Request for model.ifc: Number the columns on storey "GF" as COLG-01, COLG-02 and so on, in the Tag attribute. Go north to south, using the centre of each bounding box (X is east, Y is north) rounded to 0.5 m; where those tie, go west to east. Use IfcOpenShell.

First a look at what the model holds.

```python
import ifcopenshell
import ifcopenshell.util.element
import ifcopenshell.util.placement

model = ifcopenshell.open("model.ifc")
print(model.schema)
storey = next(s for s in model.by_type("IfcBuildingStorey") if s.Name == "GF")
columns = [e for e in ifcopenshell.util.element.get_decomposition(storey) if e.is_a("IfcColumn")]
for e in sorted(columns, key=lambda e: e.id()):
    origin = ifcopenshell.util.placement.get_local_placement(e.ObjectPlacement)[:3, 3]
    print(e.id(), e.Tag, e.Name, origin.round(2) + 0.0, sep=" | ")
```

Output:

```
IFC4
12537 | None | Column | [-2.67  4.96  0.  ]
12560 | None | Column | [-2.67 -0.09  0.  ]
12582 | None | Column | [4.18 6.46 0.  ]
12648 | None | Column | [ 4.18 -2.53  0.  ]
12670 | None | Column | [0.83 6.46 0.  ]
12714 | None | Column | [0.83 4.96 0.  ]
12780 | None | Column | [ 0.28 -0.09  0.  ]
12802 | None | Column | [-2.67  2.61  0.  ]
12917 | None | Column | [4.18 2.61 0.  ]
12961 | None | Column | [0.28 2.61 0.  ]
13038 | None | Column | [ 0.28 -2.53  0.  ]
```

```python
import ifcopenshell
import ifcopenshell.geom
import ifcopenshell.util.element
import ifcopenshell.util.shape

model = ifcopenshell.open("model.ifc")
settings = ifcopenshell.geom.settings()
settings.set("use-world-coords", True)


def centre(element):
    shape = ifcopenshell.geom.create_shape(settings, element)
    return ifcopenshell.util.shape.get_bbox_centroid(shape.geometry)


storey = next(s for s in model.by_type("IfcBuildingStorey") if s.Name == "GF")
columns = [e for e in ifcopenshell.util.element.get_decomposition(storey) if e.is_a("IfcColumn")]

# Insertion points can sit at a corner or the storey origin, so sort by the geometry (in metres).
centres = {e: centre(e) for e in columns}
columns.sort(key=lambda e: (-round(centres[e][1] / 0.5), centres[e][0]))

for i, e in enumerate(columns, start=1):
    number = f"COLG-{i:02d}"
    e.Tag = number
    print(e.id(), number)

model.write("model-out.ifc")
```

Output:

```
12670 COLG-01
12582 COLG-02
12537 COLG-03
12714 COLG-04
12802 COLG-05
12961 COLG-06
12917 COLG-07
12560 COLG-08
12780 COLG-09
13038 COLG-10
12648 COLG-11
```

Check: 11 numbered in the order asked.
